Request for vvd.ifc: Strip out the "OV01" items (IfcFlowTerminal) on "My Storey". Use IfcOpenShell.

First a look at what the model holds.

```python
import ifcopenshell
import ifcopenshell.util.element

model = ifcopenshell.open("vvd.ifc")
print(model.schema)
storey = next(s for s in model.by_type("IfcBuildingStorey") if s.Name == "My Storey")
terminals = [e for e in ifcopenshell.util.element.get_decomposition(storey) if e.is_a("IfcFlowTerminal")]
seen = {}
for e in terminals:
    element_type = ifcopenshell.util.element.get_type(e)
    name = element_type.Name if element_type not in (None, e) else None
    seen[name] = seen.get(name, 0) + 1
for name, count in sorted(seen.items(), key=str):
    print(count, "x", name)
```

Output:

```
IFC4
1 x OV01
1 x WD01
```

```python
import ifcopenshell
import ifcopenshell.api.root
import ifcopenshell.util.element

model = ifcopenshell.open("vvd.ifc")

storey = next(s for s in model.by_type("IfcBuildingStorey") if s.Name == "My Storey")
terminals = [e for e in ifcopenshell.util.element.get_decomposition(storey) if e.is_a("IfcFlowTerminal")]
targets = [e for e in terminals if (t := ifcopenshell.util.element.get_type(e)) not in (None, e) and t.Name == "OV01"]

for e in targets:
    ifcopenshell.api.root.remove_product(model, product=e)
print(len(targets), "removed")

model.write("vvd_v2.ifc")
```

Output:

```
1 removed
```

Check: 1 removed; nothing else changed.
